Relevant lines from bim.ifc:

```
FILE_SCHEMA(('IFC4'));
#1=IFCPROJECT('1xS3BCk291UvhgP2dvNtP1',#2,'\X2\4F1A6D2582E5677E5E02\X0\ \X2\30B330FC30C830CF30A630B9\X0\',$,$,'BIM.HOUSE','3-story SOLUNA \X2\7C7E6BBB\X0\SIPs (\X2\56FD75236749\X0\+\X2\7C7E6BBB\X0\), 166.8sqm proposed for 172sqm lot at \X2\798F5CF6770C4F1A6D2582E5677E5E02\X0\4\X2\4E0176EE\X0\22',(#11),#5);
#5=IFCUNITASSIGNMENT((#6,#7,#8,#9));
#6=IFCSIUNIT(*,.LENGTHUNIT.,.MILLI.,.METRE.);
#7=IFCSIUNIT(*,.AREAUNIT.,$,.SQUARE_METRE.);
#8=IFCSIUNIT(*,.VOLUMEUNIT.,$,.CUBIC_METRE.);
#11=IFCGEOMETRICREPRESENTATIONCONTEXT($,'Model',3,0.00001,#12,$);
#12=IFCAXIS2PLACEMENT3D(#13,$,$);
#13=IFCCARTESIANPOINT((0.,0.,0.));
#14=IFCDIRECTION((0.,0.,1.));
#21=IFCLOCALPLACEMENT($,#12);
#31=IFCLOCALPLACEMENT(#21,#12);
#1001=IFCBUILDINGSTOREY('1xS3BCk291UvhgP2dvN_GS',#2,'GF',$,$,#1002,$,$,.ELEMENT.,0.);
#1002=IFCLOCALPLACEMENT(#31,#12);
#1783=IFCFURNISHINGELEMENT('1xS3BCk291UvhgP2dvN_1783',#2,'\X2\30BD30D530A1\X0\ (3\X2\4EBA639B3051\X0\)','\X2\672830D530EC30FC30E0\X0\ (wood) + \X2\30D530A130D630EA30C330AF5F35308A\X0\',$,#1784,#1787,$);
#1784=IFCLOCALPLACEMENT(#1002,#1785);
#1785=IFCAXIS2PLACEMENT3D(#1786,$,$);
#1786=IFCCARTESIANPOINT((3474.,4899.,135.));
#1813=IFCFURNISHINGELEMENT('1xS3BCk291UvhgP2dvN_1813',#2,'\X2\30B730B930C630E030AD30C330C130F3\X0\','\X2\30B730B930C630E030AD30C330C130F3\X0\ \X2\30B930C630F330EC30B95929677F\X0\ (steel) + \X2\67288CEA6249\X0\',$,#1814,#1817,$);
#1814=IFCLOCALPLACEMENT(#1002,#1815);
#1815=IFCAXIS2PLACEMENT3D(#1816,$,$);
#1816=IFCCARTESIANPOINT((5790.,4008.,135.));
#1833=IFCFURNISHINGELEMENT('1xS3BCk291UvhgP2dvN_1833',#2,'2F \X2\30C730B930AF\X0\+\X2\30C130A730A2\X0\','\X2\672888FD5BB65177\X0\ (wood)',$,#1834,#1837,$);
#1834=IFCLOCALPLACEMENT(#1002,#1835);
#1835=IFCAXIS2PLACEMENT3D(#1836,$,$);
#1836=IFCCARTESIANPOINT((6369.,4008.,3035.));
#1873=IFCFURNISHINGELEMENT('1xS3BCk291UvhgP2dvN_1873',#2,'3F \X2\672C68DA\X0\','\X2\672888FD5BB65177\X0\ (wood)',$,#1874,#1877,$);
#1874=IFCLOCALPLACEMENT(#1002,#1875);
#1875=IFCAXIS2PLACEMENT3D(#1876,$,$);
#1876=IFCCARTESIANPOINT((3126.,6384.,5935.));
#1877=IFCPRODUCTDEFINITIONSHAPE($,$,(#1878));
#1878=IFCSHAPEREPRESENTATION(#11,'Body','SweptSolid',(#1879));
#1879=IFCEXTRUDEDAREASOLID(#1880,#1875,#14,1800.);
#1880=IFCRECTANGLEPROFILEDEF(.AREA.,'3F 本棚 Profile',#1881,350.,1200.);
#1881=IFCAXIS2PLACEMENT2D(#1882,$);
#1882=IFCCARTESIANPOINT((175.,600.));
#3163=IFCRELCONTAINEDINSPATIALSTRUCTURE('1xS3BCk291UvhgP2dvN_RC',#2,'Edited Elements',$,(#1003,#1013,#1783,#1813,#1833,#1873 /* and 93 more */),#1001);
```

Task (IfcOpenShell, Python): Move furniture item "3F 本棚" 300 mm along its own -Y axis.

```python
import ifcopenshell
import ifcopenshell.api.geometry
import ifcopenshell.util.placement

model = ifcopenshell.open("bim.ifc")

item = model.by_guid("1xS3BCk291UvhgP2dvN_1873")
matrix = ifcopenshell.util.placement.get_local_placement(item.ObjectPlacement)
matrix[:3, 3] -= matrix[:3, 1] * 300.0
ifcopenshell.api.geometry.edit_object_placement(model, product=item, matrix=matrix, is_si=False)

print(ifcopenshell.util.placement.get_local_placement(item.ObjectPlacement).round(3) + 0.0)

model.write("bim_updated.ifc")
```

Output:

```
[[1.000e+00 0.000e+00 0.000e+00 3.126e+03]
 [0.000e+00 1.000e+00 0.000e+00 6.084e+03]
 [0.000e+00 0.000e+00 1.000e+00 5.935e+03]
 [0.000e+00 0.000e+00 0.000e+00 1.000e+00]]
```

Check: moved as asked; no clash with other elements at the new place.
